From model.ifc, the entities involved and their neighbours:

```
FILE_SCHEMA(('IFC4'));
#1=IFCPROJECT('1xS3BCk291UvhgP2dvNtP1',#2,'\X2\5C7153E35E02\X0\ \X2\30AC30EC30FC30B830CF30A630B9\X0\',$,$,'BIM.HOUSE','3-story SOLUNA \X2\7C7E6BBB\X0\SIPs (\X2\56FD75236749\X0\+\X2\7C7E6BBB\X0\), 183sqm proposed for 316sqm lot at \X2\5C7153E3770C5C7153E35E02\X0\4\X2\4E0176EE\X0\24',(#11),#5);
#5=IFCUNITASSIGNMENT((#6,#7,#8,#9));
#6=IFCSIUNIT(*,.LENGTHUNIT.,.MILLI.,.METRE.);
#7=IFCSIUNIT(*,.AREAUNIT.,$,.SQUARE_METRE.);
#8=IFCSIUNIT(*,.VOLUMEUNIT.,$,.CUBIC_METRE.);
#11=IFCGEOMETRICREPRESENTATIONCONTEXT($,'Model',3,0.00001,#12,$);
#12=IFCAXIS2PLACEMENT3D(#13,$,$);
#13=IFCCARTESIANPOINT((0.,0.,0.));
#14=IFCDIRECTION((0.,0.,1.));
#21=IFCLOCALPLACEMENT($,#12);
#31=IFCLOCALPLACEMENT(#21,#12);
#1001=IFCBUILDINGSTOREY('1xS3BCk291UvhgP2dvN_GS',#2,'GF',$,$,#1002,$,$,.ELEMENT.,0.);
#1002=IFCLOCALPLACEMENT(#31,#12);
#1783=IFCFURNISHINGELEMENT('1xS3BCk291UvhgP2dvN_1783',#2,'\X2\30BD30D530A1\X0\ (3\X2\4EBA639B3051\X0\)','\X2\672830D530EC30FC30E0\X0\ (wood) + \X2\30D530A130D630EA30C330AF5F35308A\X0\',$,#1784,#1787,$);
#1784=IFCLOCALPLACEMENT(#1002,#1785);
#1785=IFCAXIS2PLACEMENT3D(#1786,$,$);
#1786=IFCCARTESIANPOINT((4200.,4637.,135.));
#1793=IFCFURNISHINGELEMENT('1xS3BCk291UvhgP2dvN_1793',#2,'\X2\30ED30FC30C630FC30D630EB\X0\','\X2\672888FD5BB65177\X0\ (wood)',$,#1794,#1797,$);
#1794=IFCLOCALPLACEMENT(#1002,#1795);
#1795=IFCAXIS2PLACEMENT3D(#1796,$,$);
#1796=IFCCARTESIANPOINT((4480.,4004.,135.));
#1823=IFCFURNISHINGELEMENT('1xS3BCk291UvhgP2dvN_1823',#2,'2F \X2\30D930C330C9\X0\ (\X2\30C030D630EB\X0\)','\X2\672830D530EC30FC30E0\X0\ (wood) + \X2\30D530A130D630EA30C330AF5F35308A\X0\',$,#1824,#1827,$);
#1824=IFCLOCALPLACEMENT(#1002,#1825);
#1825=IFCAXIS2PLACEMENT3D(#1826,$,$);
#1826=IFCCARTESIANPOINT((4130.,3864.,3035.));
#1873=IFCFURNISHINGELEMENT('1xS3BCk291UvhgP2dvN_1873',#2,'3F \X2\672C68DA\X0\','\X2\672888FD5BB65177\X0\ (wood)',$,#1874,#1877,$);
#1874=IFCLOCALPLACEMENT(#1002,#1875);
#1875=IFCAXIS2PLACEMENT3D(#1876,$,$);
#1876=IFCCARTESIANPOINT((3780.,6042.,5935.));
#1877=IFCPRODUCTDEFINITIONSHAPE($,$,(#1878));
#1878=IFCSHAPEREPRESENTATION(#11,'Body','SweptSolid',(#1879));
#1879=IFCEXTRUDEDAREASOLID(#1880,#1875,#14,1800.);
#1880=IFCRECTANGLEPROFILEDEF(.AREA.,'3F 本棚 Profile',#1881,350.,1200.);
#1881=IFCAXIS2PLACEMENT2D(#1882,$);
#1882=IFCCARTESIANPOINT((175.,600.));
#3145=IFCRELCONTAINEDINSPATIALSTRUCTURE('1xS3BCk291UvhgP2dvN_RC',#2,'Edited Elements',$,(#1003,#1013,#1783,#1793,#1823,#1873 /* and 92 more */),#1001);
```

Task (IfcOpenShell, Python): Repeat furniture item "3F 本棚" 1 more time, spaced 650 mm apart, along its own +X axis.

```python
import ifcopenshell
import ifcopenshell.api.geometry
import ifcopenshell.api.root
import ifcopenshell.util.element
import ifcopenshell.util.placement
import ifcopenshell.util.unit

model = ifcopenshell.open("model.ifc")
unit_scale = ifcopenshell.util.unit.calculate_unit_scale(model)


def reuse_history(source, copy):
    """copy_class also copies each property set's owner history, people and application; keep the originals."""
    for rel in copy.IsDefinedBy:
        if rel.is_a("IfcRelDefinesByProperties") and (history := rel.RelatingPropertyDefinition.OwnerHistory):
            rel.RelatingPropertyDefinition.OwnerHistory = source.OwnerHistory
            ifcopenshell.util.element.remove_deep2(model, history)


source = model.by_guid("1xS3BCk291UvhgP2dvN_1873")
base = ifcopenshell.util.placement.get_local_placement(source.ObjectPlacement)
step = base[:3, 0] * 0.65 / unit_scale

for i in range(1, 2):
    copy = ifcopenshell.api.root.copy_class(model, product=source)
    copy.Representation = ifcopenshell.util.element.copy_deep(
        model, source.Representation, exclude=["IfcGeometricRepresentationContext", "IfcRepresentationMap"]
    )
    reuse_history(source, copy)
    matrix = base.copy()
    matrix[:3, 3] += i * step
    print("added at", matrix[:3, 3].round(3) + 0.0)
    ifcopenshell.api.geometry.edit_object_placement(model, product=copy, matrix=matrix, is_si=False)

model.write("model-out.ifc")
```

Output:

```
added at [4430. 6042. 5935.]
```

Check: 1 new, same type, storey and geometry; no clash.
